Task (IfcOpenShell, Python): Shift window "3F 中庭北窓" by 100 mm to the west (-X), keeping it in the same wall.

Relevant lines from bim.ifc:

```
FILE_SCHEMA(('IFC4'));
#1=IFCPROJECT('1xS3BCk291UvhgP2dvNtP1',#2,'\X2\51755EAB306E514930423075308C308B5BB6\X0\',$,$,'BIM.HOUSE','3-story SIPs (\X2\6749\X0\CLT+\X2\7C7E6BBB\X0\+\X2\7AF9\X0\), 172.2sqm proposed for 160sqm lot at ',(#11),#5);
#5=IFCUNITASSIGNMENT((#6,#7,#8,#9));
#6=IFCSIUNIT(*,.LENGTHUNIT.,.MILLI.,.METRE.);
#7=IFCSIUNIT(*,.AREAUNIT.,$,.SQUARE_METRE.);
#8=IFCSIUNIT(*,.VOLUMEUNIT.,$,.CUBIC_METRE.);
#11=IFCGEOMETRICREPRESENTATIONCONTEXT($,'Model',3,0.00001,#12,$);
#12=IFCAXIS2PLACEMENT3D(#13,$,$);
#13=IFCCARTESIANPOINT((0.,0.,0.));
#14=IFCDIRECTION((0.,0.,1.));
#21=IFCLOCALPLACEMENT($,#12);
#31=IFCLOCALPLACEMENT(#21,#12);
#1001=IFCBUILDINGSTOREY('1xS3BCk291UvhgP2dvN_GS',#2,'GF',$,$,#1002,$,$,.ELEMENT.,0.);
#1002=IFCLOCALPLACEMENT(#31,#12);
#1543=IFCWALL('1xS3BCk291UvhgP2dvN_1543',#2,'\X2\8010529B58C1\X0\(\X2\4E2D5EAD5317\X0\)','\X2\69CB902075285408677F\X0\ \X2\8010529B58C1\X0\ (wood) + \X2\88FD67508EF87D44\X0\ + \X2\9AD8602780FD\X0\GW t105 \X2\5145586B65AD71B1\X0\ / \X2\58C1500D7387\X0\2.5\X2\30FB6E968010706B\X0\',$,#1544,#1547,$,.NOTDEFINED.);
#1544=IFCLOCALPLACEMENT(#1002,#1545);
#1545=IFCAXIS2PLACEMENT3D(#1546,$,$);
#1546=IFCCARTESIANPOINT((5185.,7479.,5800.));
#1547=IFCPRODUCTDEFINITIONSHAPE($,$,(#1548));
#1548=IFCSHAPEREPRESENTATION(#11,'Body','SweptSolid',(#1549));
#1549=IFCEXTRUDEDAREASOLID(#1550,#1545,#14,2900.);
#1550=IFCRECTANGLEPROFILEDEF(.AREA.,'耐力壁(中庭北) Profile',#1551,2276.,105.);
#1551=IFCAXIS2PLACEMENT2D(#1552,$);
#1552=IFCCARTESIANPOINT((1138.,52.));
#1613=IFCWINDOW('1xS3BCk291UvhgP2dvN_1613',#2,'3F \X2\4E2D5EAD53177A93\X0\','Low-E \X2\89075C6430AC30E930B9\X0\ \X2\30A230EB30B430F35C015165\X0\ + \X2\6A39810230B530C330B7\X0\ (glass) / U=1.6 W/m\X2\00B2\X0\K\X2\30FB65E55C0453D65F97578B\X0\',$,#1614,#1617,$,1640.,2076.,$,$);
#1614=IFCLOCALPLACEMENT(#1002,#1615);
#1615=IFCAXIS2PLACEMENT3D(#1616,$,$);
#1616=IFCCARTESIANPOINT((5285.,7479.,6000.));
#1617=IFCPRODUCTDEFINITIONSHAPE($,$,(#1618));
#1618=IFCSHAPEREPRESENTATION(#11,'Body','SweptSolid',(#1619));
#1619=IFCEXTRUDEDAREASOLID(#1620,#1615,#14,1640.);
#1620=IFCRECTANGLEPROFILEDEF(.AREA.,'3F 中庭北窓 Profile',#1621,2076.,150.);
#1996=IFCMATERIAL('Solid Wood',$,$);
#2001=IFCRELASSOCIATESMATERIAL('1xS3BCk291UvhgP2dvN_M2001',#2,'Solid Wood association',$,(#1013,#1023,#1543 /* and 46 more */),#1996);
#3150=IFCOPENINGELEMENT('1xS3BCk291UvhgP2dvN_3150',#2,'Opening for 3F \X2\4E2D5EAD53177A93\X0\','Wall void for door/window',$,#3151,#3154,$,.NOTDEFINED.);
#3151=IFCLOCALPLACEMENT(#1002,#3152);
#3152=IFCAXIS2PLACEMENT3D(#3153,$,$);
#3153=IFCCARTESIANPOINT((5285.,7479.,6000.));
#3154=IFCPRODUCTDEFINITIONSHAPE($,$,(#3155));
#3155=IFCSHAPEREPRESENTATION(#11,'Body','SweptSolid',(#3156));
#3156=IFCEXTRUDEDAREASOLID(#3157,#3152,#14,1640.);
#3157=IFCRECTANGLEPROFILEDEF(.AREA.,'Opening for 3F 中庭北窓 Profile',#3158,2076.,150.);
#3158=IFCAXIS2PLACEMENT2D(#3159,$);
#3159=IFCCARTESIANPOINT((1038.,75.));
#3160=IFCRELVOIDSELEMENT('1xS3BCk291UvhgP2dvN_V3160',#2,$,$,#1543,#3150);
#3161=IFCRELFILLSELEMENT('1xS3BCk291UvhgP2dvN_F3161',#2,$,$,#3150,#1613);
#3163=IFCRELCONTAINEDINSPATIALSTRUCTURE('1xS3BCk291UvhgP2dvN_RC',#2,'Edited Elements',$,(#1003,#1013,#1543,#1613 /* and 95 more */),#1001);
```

```python
import ifcopenshell
import ifcopenshell.api.geometry
import ifcopenshell.util.placement
import ifcopenshell.util.unit

model = ifcopenshell.open("bim.ifc")
unit_scale = ifcopenshell.util.unit.calculate_unit_scale(model)

window = model.by_guid("1xS3BCk291UvhgP2dvN_1613")
opening = window.FillsVoids[0].RelatingOpeningElement
wall = opening.VoidsElements[0].RelatingBuildingElement

wall_matrix = ifcopenshell.util.placement.get_local_placement(wall.ObjectPlacement)
shift = wall_matrix[:3, 0] * -0.1 / unit_scale
before = ifcopenshell.util.placement.get_local_placement(window.ObjectPlacement)[:3, 3].copy()

# The window is not placed relative to its opening, so move both.
for product in (opening, window):
    matrix = ifcopenshell.util.placement.get_local_placement(product.ObjectPlacement)
    matrix[:3, 3] += shift
    ifcopenshell.api.geometry.edit_object_placement(model, product=product, matrix=matrix, is_si=False)

after = ifcopenshell.util.placement.get_local_placement(window.ObjectPlacement)[:3, 3]
print("window moved by", (after - before).round(3) + 0.0)

model.write("bim_v2.ifc")
```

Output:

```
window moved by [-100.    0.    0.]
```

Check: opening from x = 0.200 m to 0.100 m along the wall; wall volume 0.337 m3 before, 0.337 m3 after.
